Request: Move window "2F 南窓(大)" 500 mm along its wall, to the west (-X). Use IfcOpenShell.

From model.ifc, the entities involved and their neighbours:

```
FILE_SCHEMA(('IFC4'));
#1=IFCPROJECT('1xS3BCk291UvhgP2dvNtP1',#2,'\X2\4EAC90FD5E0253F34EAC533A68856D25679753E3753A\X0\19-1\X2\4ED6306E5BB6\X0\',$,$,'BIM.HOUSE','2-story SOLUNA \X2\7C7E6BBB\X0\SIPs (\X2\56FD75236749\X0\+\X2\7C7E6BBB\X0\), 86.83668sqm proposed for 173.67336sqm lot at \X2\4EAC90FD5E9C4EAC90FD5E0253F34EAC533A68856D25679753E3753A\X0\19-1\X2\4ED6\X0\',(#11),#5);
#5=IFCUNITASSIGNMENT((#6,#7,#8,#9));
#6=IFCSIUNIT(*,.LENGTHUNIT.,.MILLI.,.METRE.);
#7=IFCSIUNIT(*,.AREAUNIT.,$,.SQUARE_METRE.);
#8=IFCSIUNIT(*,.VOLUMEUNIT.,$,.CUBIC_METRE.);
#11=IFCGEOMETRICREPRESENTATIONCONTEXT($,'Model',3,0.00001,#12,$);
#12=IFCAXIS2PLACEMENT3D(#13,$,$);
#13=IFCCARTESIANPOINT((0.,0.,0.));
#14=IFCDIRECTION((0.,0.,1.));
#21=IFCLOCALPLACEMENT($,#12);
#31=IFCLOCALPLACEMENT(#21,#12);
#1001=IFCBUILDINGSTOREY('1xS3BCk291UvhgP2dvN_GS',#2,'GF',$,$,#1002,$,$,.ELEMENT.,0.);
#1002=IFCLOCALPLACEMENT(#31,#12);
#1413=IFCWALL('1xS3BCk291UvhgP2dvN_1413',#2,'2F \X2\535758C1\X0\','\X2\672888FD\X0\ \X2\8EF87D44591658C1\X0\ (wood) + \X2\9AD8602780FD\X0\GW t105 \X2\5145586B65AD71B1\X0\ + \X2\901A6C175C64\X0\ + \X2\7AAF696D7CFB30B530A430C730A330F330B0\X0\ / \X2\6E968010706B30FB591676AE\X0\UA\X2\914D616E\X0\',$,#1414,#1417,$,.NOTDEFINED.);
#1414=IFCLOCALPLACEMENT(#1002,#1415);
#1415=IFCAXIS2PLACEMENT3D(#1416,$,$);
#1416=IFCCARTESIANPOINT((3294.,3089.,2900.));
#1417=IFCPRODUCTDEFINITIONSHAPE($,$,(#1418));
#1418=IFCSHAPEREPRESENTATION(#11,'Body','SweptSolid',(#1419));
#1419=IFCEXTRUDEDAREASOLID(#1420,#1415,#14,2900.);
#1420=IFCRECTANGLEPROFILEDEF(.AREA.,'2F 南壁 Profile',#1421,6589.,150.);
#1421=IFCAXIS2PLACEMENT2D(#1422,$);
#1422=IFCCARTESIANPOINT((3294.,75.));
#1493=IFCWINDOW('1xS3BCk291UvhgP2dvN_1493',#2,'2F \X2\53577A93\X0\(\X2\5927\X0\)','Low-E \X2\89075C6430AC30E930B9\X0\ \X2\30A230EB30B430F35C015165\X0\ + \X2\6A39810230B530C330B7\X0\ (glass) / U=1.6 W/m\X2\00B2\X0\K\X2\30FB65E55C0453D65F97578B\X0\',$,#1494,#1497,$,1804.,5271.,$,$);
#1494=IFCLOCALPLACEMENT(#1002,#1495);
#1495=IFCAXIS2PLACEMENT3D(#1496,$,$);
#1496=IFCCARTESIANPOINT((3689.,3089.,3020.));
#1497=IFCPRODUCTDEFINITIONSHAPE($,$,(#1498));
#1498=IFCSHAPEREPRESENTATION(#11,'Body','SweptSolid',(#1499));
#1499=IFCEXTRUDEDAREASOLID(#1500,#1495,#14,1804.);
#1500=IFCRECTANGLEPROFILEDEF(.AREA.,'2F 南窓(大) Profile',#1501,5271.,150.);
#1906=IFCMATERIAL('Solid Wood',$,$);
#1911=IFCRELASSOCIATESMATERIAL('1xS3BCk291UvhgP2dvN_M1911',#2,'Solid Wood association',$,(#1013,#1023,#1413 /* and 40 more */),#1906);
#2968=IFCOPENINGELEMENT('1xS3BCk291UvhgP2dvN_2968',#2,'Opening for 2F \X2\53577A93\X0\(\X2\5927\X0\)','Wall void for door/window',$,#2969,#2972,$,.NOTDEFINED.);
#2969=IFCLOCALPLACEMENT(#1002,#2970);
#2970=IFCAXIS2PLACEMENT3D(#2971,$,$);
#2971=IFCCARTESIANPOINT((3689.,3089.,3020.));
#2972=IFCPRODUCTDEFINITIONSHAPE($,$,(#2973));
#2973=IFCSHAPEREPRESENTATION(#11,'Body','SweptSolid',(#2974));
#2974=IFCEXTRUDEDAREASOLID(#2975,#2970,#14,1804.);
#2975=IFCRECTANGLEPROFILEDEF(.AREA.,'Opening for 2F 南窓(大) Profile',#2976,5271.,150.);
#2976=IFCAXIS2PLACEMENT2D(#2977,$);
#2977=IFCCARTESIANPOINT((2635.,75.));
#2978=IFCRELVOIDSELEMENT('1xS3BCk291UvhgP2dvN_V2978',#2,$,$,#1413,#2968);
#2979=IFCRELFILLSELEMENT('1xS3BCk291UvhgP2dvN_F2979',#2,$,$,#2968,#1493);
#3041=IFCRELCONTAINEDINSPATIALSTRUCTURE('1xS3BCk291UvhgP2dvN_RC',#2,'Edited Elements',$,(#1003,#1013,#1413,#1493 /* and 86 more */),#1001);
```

```python
import ifcopenshell
import ifcopenshell.api.geometry
import ifcopenshell.util.placement

model = ifcopenshell.open("model.ifc")

window = model.by_guid("1xS3BCk291UvhgP2dvN_1493")
opening = window.FillsVoids[0].RelatingOpeningElement
wall = opening.VoidsElements[0].RelatingBuildingElement

wall_matrix = ifcopenshell.util.placement.get_local_placement(wall.ObjectPlacement)
shift = wall_matrix[:3, 0] * -500.0
before = ifcopenshell.util.placement.get_local_placement(window.ObjectPlacement)[:3, 3].copy()

# The window is not placed relative to its opening, so move both.
for product in (opening, window):
    matrix = ifcopenshell.util.placement.get_local_placement(product.ObjectPlacement)
    matrix[:3, 3] += shift
    ifcopenshell.api.geometry.edit_object_placement(model, product=product, matrix=matrix, is_si=False)

after = ifcopenshell.util.placement.get_local_placement(window.ObjectPlacement)[:3, 3]
print("window moved by", (after - before).round(3) + 0.0)

model.write("model_updated.ifc")
```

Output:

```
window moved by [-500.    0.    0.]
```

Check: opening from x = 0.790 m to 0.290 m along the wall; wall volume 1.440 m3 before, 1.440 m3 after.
